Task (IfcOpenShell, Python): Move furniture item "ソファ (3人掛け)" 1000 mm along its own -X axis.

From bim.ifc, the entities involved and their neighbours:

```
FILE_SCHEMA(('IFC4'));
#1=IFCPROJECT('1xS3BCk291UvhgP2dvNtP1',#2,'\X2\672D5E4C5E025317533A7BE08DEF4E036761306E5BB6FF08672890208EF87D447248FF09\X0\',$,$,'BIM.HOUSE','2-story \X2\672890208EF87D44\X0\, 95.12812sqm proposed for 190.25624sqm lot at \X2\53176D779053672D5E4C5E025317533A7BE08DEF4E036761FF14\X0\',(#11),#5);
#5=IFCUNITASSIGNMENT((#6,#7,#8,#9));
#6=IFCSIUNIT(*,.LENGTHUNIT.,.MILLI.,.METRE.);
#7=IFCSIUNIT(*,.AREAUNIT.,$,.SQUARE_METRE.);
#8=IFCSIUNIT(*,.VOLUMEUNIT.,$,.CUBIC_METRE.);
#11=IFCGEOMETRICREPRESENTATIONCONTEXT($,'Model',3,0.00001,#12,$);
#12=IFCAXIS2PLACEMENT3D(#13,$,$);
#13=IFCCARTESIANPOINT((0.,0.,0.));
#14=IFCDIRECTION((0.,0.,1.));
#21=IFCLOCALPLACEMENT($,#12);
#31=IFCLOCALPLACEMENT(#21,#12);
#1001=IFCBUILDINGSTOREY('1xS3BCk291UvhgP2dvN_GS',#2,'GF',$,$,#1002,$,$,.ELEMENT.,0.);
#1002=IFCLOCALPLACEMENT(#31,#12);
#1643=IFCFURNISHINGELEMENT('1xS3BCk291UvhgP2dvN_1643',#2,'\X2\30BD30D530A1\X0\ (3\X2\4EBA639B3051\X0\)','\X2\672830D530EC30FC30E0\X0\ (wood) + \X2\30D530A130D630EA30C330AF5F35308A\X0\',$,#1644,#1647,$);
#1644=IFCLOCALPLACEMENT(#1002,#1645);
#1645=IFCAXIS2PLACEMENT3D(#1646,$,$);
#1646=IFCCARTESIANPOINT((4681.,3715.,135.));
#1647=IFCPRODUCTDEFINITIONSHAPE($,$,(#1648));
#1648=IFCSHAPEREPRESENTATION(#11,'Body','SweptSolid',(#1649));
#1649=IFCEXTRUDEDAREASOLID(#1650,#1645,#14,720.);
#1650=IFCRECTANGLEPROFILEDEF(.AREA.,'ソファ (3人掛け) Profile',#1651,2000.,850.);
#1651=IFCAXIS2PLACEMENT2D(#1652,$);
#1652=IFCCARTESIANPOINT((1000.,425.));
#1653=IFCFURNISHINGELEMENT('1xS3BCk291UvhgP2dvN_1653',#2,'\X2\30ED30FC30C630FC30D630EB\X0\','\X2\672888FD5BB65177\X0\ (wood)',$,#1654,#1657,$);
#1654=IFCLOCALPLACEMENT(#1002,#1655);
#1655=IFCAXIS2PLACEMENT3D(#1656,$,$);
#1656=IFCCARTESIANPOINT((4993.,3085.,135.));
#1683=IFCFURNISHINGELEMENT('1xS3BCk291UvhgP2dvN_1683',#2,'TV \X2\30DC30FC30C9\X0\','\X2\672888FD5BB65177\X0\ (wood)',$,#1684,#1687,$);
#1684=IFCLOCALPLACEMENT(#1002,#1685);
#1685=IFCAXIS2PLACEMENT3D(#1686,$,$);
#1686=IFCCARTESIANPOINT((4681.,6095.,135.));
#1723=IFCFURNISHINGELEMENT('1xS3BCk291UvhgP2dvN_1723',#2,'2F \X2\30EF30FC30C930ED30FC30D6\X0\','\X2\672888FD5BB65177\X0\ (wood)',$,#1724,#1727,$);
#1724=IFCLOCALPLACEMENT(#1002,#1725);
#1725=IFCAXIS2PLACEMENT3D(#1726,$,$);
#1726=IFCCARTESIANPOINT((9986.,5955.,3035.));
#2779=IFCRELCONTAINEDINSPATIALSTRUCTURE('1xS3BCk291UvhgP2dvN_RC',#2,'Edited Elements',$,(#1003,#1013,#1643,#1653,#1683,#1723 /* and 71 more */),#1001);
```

```python
import ifcopenshell
import ifcopenshell.api.geometry
import ifcopenshell.util.placement
import ifcopenshell.util.unit

model = ifcopenshell.open("bim.ifc")
unit_scale = ifcopenshell.util.unit.calculate_unit_scale(model)

item = model.by_id(1643)
matrix = ifcopenshell.util.placement.get_local_placement(item.ObjectPlacement)
matrix[:3, 3] -= matrix[:3, 0] * 1 / unit_scale
ifcopenshell.api.geometry.edit_object_placement(model, product=item, matrix=matrix, is_si=False)

print(ifcopenshell.util.placement.get_local_placement(item.ObjectPlacement).round(3) + 0.0)

model.write("bim_edited.ifc")
```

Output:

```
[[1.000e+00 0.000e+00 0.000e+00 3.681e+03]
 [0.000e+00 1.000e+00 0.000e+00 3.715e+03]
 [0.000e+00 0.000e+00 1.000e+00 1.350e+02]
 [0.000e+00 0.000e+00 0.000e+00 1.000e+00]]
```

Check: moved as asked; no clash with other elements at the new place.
